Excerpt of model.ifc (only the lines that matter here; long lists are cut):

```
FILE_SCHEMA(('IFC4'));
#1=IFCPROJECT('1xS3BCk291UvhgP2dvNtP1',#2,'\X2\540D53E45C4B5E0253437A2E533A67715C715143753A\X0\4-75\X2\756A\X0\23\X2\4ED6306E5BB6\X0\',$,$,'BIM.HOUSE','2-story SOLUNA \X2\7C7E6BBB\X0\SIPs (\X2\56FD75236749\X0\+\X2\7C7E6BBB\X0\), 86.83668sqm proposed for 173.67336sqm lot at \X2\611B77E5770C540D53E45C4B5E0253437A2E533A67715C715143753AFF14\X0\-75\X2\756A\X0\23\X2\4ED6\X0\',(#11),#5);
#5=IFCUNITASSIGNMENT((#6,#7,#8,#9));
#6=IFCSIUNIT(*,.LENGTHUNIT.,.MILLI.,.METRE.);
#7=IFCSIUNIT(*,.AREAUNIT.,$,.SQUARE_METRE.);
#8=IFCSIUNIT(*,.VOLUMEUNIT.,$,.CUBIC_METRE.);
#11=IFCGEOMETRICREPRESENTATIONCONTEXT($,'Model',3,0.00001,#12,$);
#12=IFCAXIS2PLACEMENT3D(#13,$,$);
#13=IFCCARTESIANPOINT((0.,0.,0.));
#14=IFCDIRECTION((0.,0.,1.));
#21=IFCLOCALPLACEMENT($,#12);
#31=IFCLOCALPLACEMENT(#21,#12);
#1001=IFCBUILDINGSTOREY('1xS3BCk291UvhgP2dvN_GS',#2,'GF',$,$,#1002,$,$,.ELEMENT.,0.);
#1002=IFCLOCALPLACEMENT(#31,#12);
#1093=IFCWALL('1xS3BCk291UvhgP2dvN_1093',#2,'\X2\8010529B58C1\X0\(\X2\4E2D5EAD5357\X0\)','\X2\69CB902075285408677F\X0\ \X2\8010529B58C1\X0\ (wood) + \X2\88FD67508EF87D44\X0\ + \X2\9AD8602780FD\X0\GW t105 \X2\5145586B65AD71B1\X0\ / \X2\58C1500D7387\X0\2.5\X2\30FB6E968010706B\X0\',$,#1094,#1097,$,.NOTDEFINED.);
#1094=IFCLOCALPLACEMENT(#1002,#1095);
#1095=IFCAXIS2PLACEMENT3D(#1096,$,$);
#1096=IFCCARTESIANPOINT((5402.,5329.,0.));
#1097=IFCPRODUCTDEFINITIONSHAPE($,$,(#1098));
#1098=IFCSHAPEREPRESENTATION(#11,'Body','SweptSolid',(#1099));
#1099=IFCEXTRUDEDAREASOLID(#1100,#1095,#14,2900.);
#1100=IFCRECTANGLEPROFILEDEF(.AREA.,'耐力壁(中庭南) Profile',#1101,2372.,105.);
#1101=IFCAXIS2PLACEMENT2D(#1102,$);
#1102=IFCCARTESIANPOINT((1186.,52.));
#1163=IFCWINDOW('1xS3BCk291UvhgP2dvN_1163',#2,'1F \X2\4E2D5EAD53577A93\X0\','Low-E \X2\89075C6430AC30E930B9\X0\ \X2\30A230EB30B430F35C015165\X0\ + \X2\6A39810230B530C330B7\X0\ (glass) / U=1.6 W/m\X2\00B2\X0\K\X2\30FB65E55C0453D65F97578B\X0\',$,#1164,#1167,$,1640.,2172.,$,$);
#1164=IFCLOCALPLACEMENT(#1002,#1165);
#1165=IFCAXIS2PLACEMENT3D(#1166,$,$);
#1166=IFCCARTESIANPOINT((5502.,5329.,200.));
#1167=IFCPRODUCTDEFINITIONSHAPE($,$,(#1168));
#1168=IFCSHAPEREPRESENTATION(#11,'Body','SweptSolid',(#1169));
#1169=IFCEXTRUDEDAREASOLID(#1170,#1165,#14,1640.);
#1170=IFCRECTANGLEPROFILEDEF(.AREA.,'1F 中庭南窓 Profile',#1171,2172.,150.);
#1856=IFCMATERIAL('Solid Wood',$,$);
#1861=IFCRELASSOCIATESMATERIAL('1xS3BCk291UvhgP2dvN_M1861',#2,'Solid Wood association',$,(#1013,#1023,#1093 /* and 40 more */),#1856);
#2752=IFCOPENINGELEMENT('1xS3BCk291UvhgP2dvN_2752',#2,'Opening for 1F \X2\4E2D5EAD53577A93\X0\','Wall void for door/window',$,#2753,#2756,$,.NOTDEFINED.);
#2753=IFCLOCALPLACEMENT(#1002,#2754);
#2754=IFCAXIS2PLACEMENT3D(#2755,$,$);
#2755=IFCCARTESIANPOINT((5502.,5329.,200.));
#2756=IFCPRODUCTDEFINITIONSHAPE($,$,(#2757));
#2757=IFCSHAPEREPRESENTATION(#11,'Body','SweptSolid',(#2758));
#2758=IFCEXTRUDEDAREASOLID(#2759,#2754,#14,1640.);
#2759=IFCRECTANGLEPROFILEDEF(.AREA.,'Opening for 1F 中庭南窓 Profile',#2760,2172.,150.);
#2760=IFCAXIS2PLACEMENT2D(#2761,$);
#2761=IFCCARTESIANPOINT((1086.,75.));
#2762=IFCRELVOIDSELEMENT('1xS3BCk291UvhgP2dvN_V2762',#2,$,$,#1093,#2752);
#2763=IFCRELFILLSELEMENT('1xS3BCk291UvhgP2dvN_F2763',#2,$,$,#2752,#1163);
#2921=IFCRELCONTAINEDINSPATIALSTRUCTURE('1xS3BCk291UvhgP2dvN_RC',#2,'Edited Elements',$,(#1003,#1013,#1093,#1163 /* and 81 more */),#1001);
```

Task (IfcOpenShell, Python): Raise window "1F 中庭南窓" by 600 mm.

```python
import numpy as np
import ifcopenshell
import ifcopenshell.api.geometry
import ifcopenshell.util.placement
import ifcopenshell.util.unit

model = ifcopenshell.open("model.ifc")
unit_scale = ifcopenshell.util.unit.calculate_unit_scale(model)

window = model.by_guid("1xS3BCk291UvhgP2dvN_1163")
opening = window.FillsVoids[0].RelatingOpeningElement
dz = 0.6 / unit_scale

shift = np.array([0.0, 0.0, dz])
# The window is not placed relative to its opening, so move both.
for product in (opening, window):
    matrix = ifcopenshell.util.placement.get_local_placement(product.ObjectPlacement)
    matrix[:3, 3] += shift
    ifcopenshell.api.geometry.edit_object_placement(model, product=product, matrix=matrix, is_si=False)

print(f"moved by {dz * unit_scale:+.3f} m")

model.write("model_rev.ifc")
```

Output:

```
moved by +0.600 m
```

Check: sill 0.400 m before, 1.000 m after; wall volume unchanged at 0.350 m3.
